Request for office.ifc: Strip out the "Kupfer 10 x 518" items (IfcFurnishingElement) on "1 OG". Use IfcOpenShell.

First a look at what the model holds.

```python
import ifcopenshell
import ifcopenshell.util.element

model = ifcopenshell.open("office.ifc")
print(model.schema)
storey = next(s for s in model.by_type("IfcBuildingStorey") if s.Name == "1 OG")
furniture = [e for e in ifcopenshell.util.element.get_decomposition(storey) if e.is_a("IfcFurnishingElement")]
seen = {}
for e in furniture:
    element_type = ifcopenshell.util.element.get_type(e)
    name = element_type.Name if element_type not in (None, e) else None
    seen[name] = seen.get(name, 0) + 1
for name, count in sorted(seen.items(), key=str):
    print(count, "x", name)
```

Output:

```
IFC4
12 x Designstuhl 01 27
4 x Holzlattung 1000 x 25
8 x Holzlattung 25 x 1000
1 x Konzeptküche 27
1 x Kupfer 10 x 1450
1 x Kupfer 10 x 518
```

```python
import ifcopenshell
import ifcopenshell.api.root
import ifcopenshell.util.element

model = ifcopenshell.open("office.ifc")

storey = next(s for s in model.by_type("IfcBuildingStorey") if s.Name == "1 OG")
furniture = [e for e in ifcopenshell.util.element.get_decomposition(storey) if e.is_a("IfcFurnishingElement")]
targets = [e for e in furniture if (t := ifcopenshell.util.element.get_type(e)) not in (None, e) and t.Name == "Kupfer 10 x 518"]

for e in targets:
    ifcopenshell.api.root.remove_product(model, product=e)
print(len(targets), "removed")

model.write("office_updated.ifc")
```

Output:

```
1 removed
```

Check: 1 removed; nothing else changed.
